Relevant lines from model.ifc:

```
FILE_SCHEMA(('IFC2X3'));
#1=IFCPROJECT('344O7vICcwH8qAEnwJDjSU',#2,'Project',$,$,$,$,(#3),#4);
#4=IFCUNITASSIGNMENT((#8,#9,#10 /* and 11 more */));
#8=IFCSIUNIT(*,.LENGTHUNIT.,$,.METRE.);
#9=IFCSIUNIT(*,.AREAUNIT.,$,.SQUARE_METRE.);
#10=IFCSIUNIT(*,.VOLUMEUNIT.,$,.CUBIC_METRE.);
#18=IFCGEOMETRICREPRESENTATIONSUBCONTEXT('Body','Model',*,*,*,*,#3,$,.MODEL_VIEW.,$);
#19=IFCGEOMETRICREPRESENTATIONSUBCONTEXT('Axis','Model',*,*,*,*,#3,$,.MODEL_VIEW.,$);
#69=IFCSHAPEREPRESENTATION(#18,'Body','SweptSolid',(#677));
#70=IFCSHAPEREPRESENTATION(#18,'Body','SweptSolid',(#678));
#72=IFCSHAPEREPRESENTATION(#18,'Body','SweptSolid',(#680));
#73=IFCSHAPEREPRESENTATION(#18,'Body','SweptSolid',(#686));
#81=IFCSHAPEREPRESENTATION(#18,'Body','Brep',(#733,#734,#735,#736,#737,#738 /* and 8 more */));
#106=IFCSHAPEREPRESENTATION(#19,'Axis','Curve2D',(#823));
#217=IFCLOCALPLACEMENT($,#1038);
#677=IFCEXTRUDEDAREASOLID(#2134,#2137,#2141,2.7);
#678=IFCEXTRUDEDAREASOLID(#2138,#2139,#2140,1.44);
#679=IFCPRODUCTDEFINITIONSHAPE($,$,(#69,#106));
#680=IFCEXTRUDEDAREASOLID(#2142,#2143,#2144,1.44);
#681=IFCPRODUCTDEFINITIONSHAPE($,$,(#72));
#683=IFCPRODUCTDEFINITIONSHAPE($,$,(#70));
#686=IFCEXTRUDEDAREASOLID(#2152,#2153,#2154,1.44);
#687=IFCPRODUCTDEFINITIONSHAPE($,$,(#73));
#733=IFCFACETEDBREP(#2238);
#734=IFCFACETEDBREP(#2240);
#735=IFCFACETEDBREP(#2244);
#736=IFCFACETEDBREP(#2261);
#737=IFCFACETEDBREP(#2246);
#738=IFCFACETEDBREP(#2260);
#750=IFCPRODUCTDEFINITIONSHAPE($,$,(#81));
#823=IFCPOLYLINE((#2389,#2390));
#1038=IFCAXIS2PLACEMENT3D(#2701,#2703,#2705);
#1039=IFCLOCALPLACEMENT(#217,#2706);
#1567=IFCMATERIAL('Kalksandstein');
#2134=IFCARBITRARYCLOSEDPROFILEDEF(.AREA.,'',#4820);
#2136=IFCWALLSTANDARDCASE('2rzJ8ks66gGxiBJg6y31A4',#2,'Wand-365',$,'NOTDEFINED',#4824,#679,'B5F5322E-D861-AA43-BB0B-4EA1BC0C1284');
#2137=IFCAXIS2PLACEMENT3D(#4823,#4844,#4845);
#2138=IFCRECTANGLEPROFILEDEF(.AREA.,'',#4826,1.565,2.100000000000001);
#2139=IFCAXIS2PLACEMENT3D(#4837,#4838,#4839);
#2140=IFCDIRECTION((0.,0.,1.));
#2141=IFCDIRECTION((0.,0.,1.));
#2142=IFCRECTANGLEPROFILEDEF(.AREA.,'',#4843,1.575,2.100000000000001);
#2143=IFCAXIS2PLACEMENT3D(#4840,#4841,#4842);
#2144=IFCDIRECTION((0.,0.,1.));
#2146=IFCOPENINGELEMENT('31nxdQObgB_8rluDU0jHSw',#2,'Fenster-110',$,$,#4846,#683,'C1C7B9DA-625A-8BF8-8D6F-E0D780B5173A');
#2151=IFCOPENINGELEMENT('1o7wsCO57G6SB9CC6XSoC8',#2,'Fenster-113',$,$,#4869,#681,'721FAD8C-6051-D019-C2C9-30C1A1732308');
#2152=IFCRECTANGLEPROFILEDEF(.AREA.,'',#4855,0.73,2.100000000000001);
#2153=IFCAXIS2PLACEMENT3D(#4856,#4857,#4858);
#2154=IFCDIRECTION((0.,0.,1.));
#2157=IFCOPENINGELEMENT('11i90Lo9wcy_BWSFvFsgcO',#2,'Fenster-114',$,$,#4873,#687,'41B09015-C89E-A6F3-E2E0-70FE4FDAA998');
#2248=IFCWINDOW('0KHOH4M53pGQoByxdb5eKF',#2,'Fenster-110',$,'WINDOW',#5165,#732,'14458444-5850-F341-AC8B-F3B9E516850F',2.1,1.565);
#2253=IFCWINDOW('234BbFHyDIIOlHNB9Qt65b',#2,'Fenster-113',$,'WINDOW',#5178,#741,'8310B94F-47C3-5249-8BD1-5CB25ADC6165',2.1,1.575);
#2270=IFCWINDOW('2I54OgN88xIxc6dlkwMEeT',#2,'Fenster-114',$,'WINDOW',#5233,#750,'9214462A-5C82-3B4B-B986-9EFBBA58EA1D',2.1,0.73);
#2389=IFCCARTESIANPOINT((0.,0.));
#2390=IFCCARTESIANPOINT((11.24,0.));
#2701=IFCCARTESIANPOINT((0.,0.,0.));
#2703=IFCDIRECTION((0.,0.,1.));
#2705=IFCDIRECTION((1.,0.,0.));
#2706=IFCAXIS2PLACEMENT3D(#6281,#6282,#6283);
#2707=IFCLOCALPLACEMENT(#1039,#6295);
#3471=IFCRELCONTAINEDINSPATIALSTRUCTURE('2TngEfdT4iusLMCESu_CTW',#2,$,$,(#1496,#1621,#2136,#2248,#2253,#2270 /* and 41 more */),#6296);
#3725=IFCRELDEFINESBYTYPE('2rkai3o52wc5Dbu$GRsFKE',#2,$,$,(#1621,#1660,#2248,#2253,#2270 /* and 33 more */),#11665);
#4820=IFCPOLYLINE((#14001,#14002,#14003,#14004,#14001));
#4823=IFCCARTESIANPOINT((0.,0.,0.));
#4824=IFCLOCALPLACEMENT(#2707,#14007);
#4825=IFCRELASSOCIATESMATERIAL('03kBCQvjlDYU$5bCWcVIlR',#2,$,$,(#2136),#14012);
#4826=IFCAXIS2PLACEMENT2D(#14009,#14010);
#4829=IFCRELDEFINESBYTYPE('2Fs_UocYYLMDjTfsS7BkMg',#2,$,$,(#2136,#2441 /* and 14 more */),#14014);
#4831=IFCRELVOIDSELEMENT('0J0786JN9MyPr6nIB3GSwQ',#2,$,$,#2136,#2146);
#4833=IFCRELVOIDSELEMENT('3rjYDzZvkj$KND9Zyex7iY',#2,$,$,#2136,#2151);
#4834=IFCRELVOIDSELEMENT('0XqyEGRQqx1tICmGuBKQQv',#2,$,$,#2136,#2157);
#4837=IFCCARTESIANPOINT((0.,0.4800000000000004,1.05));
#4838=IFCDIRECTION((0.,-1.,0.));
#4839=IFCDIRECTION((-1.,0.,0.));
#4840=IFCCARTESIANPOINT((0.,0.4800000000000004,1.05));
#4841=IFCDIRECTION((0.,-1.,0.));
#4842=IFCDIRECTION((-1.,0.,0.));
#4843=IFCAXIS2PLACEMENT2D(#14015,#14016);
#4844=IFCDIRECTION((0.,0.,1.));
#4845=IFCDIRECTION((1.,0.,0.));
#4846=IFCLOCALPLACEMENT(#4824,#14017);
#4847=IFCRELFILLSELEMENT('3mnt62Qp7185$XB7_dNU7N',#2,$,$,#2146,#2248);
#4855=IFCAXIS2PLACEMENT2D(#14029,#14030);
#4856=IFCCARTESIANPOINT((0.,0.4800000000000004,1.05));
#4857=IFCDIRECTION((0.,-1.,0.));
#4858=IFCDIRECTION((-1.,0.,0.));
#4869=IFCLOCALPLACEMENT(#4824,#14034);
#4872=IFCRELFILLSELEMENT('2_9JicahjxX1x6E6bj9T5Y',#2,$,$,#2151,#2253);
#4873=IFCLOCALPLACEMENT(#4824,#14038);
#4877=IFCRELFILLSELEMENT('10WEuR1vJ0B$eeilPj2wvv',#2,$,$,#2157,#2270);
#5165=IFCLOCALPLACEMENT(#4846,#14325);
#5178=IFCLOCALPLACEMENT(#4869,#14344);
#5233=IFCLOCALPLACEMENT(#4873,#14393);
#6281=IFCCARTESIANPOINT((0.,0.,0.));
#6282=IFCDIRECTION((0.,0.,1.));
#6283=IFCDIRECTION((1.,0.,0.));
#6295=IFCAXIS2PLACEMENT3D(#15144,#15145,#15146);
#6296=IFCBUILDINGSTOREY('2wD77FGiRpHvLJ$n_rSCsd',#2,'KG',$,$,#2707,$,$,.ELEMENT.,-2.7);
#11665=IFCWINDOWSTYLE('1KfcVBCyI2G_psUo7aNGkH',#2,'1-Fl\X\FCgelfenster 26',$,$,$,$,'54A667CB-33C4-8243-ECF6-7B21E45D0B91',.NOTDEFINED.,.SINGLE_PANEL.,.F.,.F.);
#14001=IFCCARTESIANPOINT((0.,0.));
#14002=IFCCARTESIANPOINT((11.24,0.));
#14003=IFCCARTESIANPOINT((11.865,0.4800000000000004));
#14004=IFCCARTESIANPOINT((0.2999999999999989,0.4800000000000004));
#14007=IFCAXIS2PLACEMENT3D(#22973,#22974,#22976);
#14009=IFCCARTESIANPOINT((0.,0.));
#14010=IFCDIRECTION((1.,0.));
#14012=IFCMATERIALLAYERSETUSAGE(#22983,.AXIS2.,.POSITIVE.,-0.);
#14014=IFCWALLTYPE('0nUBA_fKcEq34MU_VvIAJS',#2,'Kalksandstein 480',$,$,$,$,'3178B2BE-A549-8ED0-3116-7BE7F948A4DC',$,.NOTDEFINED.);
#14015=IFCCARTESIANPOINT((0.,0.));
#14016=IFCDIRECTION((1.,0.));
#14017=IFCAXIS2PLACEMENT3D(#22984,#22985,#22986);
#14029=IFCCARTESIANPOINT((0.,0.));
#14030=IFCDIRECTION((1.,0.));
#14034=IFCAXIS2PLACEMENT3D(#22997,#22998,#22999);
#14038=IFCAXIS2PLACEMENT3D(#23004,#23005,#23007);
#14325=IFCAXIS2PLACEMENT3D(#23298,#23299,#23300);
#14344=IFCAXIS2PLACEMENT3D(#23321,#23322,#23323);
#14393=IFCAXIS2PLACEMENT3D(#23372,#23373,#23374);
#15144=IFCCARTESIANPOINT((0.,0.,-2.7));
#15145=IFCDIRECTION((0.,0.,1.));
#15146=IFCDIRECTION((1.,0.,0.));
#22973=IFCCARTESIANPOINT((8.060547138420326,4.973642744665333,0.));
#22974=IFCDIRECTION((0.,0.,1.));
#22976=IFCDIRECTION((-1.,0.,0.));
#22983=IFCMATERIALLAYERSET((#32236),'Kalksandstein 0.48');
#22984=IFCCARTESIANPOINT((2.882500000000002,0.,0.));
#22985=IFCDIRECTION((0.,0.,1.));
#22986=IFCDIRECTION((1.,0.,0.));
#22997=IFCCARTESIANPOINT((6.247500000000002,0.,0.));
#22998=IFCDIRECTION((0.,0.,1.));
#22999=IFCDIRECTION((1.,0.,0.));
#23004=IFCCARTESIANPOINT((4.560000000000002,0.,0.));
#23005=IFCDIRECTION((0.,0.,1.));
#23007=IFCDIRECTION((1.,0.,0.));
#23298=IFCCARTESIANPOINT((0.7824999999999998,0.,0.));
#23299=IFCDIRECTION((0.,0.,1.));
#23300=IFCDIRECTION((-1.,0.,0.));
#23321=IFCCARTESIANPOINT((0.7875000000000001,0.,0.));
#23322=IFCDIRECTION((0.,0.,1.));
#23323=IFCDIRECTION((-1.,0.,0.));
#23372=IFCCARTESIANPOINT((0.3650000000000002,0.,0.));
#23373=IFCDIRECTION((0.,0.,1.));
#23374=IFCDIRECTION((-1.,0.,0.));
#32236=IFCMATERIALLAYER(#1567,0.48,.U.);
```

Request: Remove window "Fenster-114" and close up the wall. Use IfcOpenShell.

```python
import ifcopenshell
import ifcopenshell.api.feature
import ifcopenshell.api.root
import ifcopenshell.geom
import ifcopenshell.util.shape

model = ifcopenshell.open("model.ifc")
settings = ifcopenshell.geom.settings()


def volume(element):
    """Net volume in cubic metres, openings subtracted."""
    shape = ifcopenshell.geom.create_shape(settings, element)
    return ifcopenshell.util.shape.get_volume(shape.geometry)


window = model.by_guid("2I54OgN88xIxc6dlkwMEeT")
opening = window.FillsVoids[0].RelatingOpeningElement
wall = opening.VoidsElements[0].RelatingBuildingElement
before = volume(wall)

ifcopenshell.api.root.remove_product(model, product=window)
ifcopenshell.api.feature.remove_feature(model, feature=opening)

after = volume(wall)

print(f"wall volume {before:.3f} -> {after:.3f} m3")

model.write("model_edited.ifc")
```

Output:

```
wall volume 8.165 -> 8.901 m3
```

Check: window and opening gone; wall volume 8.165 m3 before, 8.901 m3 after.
